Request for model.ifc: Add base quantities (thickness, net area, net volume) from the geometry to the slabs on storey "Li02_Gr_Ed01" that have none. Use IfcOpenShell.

First a look at what the model holds.

```python
import ifcopenshell
import ifcopenshell.util.element
import ifcopenshell.util.unit

model = ifcopenshell.open("model.ifc")
print(model.schema)
for unit_type in ("LENGTHUNIT", "AREAUNIT", "VOLUMEUNIT"):
    print(unit_type, ifcopenshell.util.unit.calculate_unit_scale(model, unit_type))
storey = next(s for s in model.by_type("IfcBuildingStorey") if s.Name == "Li02_Gr_Ed01")
slabs = [e for e in ifcopenshell.util.element.get_decomposition(storey) if e.is_a("IfcSlab")]
for e in sorted(slabs, key=lambda e: e.id()):
    print(e.id(), e.is_a(), e.Name, list(ifcopenshell.util.element.get_psets(e, qtos_only=True)), sep=" | ")
```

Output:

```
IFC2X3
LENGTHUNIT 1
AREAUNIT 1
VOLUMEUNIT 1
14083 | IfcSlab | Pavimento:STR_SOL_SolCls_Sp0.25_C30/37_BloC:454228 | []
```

```python
import ifcopenshell
import ifcopenshell.api.pset
import ifcopenshell.geom
import ifcopenshell.util.element
import ifcopenshell.util.shape
import ifcopenshell.util.unit

model = ifcopenshell.open("model.ifc")
unit_scale = ifcopenshell.util.unit.calculate_unit_scale(model)
area_scale = ifcopenshell.util.unit.calculate_unit_scale(model, "AREAUNIT")
volume_scale = ifcopenshell.util.unit.calculate_unit_scale(model, "VOLUMEUNIT")
settings = ifcopenshell.geom.settings()

storey = next(s for s in model.by_type("IfcBuildingStorey") if s.Name == "Li02_Gr_Ed01")
slabs = [e for e in ifcopenshell.util.element.get_decomposition(storey) if e.is_a("IfcSlab")]

for e in sorted(slabs, key=lambda e: e.id()):
    if ifcopenshell.util.element.get_psets(e, qtos_only=True, should_inherit=False):
        continue
    # Geometry comes back in metres, in the element's own axes.
    shape = ifcopenshell.geom.create_shape(settings, e)
    values = {
        "Width": ifcopenshell.util.shape.get_z(shape.geometry) / unit_scale,
        "NetArea": ifcopenshell.util.shape.get_footprint_area(shape.geometry) / area_scale,
        "NetVolume": ifcopenshell.util.shape.get_volume(shape.geometry) / volume_scale,
    }
    qto = ifcopenshell.api.pset.add_qto(model, product=e, name="BaseQuantities")
    ifcopenshell.api.pset.edit_qto(model, qto=qto, properties=values)
    print(e.id(), {k: round(v, 3) for k, v in values.items()})

model.write("model-out.ifc")
```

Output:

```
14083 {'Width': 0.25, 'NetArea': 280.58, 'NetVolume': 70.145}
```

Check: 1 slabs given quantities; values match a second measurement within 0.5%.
